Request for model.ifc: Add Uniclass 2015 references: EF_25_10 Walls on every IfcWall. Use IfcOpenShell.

First a look at what the model holds.

```python
import ifcopenshell

model = ifcopenshell.open("model.ifc")
print(model.schema)
print("classifications:", [c.Name for c in model.by_type("IfcClassification")])
for ifc_class in ("IfcDoor", "IfcRoof", "IfcStair", "IfcWall", "IfcWindow"):
    print(ifc_class, len(model.by_type(ifc_class)))
```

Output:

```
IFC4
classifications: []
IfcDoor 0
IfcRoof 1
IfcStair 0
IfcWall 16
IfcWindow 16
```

```python
import ifcopenshell
import ifcopenshell.api.classification

model = ifcopenshell.open("model.ifc")

system = ifcopenshell.api.classification.add_classification(model, classification="Uniclass 2015")

codes = {
    "IfcWall": ("EF_25_10", "Walls"),
}
for ifc_class, (code, name) in codes.items():
    products = model.by_type(ifc_class)
    ifcopenshell.api.classification.add_reference(
        model, products=products, classification=system, identification=code, name=name
    )
    print(code, len(products))

model.write("model_v2.ifc")
```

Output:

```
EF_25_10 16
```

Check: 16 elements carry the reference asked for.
